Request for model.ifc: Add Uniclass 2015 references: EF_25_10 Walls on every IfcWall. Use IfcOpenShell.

First a look at what the model holds.

```python
import ifcopenshell

model = ifcopenshell.open("model.ifc")
print(model.schema)
print("classifications:", [c.Name for c in model.by_type("IfcClassification")])
for ifc_class in ("IfcDoor", "IfcRoof", "IfcStair", "IfcWall", "IfcWindow"):
    print(ifc_class, len(model.by_type(ifc_class)))
```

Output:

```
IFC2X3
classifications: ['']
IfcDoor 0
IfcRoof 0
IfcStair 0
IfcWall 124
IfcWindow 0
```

```python
import ifcopenshell
import ifcopenshell.api.classification

model = ifcopenshell.open("model.ifc")

# IFC2X3 requires Source and Edition and has no link from the project to the system.
system = model.create_entity("IfcClassification", Source="NBS", Edition="2015", Name="Uniclass 2015")

codes = {
    "IfcWall": ("EF_25_10", "Walls"),
}
for ifc_class, (code, name) in codes.items():
    products = model.by_type(ifc_class)
    ifcopenshell.api.classification.add_reference(
        model, products=products, classification=system, identification=code, name=name
    )
    print(code, len(products))

model.write("model_rev.ifc")
```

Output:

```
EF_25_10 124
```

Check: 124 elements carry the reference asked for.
